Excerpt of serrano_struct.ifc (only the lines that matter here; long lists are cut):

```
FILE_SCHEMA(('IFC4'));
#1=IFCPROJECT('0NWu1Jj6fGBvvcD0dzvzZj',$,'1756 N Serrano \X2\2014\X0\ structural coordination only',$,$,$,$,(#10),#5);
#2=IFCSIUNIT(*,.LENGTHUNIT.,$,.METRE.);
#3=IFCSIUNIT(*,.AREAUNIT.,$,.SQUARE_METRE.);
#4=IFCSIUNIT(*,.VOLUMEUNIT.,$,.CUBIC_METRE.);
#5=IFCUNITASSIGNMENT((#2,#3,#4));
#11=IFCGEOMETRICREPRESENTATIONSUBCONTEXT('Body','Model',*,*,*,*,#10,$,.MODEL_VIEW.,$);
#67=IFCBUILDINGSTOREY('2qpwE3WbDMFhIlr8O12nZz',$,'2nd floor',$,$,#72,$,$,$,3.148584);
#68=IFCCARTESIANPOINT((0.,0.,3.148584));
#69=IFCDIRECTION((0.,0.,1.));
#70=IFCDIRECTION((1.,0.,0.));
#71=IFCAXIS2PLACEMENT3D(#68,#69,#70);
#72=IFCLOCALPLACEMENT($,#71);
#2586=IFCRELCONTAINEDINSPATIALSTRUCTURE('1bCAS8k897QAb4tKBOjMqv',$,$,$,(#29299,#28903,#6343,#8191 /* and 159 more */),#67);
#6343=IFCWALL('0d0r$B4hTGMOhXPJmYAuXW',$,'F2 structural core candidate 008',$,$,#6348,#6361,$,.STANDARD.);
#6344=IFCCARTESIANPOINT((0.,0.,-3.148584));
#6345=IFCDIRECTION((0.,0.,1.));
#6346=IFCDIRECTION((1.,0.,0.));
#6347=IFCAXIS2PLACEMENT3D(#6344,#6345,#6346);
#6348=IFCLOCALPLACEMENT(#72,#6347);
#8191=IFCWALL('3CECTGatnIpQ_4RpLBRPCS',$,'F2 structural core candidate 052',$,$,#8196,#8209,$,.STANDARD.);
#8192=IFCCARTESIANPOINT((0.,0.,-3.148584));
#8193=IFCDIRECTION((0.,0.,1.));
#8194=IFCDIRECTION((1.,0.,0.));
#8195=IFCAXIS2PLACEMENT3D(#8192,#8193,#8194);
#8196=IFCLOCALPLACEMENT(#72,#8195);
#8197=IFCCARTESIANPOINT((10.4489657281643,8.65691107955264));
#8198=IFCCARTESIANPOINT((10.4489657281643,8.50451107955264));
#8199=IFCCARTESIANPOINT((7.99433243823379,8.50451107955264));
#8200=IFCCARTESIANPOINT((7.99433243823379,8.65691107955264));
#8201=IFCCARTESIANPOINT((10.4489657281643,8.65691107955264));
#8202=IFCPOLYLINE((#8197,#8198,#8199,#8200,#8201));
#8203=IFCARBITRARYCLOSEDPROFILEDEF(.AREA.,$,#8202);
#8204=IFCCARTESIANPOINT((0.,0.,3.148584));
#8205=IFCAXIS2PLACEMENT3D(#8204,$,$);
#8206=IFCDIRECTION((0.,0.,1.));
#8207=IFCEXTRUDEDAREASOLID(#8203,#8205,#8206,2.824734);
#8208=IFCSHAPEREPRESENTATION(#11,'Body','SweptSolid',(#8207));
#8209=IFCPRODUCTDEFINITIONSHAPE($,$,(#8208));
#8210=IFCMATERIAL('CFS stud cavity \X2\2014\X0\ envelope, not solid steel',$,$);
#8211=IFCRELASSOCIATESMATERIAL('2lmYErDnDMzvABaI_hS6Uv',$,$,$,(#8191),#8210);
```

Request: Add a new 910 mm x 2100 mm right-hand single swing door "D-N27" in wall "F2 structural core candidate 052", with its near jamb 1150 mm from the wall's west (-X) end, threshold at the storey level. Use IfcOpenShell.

```python
import numpy as np
import ifcopenshell
import ifcopenshell.api.feature
import ifcopenshell.api.geometry
import ifcopenshell.api.root
import ifcopenshell.api.spatial
import ifcopenshell.geom
import ifcopenshell.util.element
import ifcopenshell.util.placement
import ifcopenshell.util.representation
import ifcopenshell.util.shape
import ifcopenshell.util.unit

model = ifcopenshell.open("serrano_struct.ifc")
unit_scale = ifcopenshell.util.unit.calculate_unit_scale(model)
settings = ifcopenshell.geom.settings()


def volume(element):
    """Net volume in cubic metres, openings subtracted."""
    shape = ifcopenshell.geom.create_shape(settings, element)
    return ifcopenshell.util.shape.get_volume(shape.geometry)


wall = model.by_guid("3CECTGatnIpQ_4RpLBRPCS")
storey = ifcopenshell.util.element.get_container(wall, ifc_class="IfcBuildingStorey")
context = ifcopenshell.util.representation.get_context(model, "Model", "Body", "MODEL_VIEW")
before = volume(wall)

width, height, from_end, sill = 0.91, 2.1, 1.15, 0.0  # metres

# The wall runs along its own X axis, and the end named is its -X end.
wall_shape = ifcopenshell.geom.create_shape(settings, wall)
x, y, z = ifcopenshell.util.shape.get_vertices(wall_shape.geometry).T
start = x.min() + from_end
face, thickness = float(y.min()), float(y.max() - y.min())
wall_matrix = ifcopenshell.util.placement.get_local_placement(wall.ObjectPlacement)
level = ifcopenshell.util.placement.get_local_placement(storey.ObjectPlacement)[2, 3]


def in_wall(x, y):
    """Placement at x, y metres in the wall's axes, at sill height."""
    matrix = wall_matrix.copy()
    matrix[:, 3] = wall_matrix @ np.array([x / unit_scale, y / unit_scale, 0.0, 1.0])
    matrix[2, 3] = level + sill / unit_scale
    return matrix


# Opening: a box that overshoots both wall faces by 50 mm.
opening = ifcopenshell.api.root.create_entity(model, ifc_class="IfcOpeningElement", predefined_type="OPENING")
box = ifcopenshell.api.geometry.add_wall_representation(
    model, context=context, length=width, height=height, thickness=thickness + 0.1
)
ifcopenshell.api.geometry.assign_representation(model, product=opening, representation=box)
ifcopenshell.api.geometry.edit_object_placement(model, product=opening, matrix=in_wall(start, face - 0.05), is_si=False)
ifcopenshell.api.feature.add_feature(model, feature=opening, element=wall)

door = ifcopenshell.api.root.create_entity(model, ifc_class="IfcDoor", name="D-N27", predefined_type="DOOR")
door.OverallWidth, door.OverallHeight = width / unit_scale, height / unit_scale
door.OperationType = "SINGLE_SWING_RIGHT"
body = ifcopenshell.api.geometry.add_door_representation(
    model,
    context=context,
    overall_width=door.OverallWidth,
    overall_height=door.OverallHeight,
    operation_type="SINGLE_SWING_RIGHT",
    lining_properties={"LiningDepth": thickness / unit_scale, "ThresholdDepth": thickness / unit_scale},
)
ifcopenshell.api.geometry.assign_representation(model, product=door, representation=body)
ifcopenshell.api.spatial.assign_container(model, products=[door], relating_structure=storey)
ifcopenshell.api.feature.add_filling(model, opening=opening, element=door)

# The lining spans the wall, so the door starts at the wall face.
ifcopenshell.api.geometry.edit_object_placement(model, product=door, matrix=in_wall(start, face), is_si=False)

after = volume(wall)

print(f"wall volume {before:.3f} -> {after:.3f} m3")

model.write("serrano_struct_edited.ifc")
```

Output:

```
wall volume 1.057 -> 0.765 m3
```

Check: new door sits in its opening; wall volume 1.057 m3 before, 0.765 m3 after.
